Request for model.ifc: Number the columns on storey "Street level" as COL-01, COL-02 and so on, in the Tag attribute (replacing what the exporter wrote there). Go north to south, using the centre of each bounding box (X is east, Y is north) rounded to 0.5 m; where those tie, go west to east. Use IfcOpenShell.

First a look at what the model holds.

```python
import ifcopenshell
import ifcopenshell.util.element
import ifcopenshell.util.placement

model = ifcopenshell.open("model.ifc")
print(model.schema)
storey = next(s for s in model.by_type("IfcBuildingStorey") if s.Name == "Street level")
columns = [e for e in ifcopenshell.util.element.get_decomposition(storey) if e.is_a("IfcColumn")]
for e in sorted(columns, key=lambda e: e.id()):
    origin = ifcopenshell.util.placement.get_local_placement(e.ObjectPlacement)[:3, 3]
    print(e.id(), e.Tag, e.Name, origin.round(2) + 0.0, sep=" | ")
```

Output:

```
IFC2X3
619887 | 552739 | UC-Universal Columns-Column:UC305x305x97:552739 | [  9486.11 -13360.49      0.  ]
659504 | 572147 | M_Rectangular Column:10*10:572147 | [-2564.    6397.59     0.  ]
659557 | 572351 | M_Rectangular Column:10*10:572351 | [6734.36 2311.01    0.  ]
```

```python
import ifcopenshell
import ifcopenshell.geom
import ifcopenshell.util.element
import ifcopenshell.util.shape

model = ifcopenshell.open("model.ifc")
settings = ifcopenshell.geom.settings()
settings.set("use-world-coords", True)


def centre(element):
    shape = ifcopenshell.geom.create_shape(settings, element)
    return ifcopenshell.util.shape.get_bbox_centroid(shape.geometry)


storey = next(s for s in model.by_type("IfcBuildingStorey") if s.Name == "Street level")
columns = [e for e in ifcopenshell.util.element.get_decomposition(storey) if e.is_a("IfcColumn")]

# Insertion points can sit at a corner or the storey origin, so sort by the geometry (in metres).
centres = {e: centre(e) for e in columns}
columns.sort(key=lambda e: (-round(centres[e][1] / 0.5), centres[e][0]))

for i, e in enumerate(columns, start=1):
    number = f"COL-{i:02d}"
    e.Tag = number
    print(e.id(), number)

model.write("model-out.ifc")
```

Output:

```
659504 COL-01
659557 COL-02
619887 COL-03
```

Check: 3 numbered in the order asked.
